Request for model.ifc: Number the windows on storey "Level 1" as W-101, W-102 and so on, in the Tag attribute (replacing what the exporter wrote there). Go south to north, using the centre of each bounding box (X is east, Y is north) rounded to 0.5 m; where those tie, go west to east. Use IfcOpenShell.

First a look at what the model holds.

```python
import ifcopenshell
import ifcopenshell.util.element
import ifcopenshell.util.placement

model = ifcopenshell.open("model.ifc")
print(model.schema)
storey = next(s for s in model.by_type("IfcBuildingStorey") if s.Name == "Level 1")
windows = [e for e in ifcopenshell.util.element.get_decomposition(storey) if e.is_a("IfcWindow")]
for e in sorted(windows, key=lambda e: e.id()):
    origin = ifcopenshell.util.placement.get_local_placement(e.ObjectPlacement)[:3, 3]
    print(e.id(), e.Tag, e.Name, origin.round(2) + 0.0, sep=" | ")
```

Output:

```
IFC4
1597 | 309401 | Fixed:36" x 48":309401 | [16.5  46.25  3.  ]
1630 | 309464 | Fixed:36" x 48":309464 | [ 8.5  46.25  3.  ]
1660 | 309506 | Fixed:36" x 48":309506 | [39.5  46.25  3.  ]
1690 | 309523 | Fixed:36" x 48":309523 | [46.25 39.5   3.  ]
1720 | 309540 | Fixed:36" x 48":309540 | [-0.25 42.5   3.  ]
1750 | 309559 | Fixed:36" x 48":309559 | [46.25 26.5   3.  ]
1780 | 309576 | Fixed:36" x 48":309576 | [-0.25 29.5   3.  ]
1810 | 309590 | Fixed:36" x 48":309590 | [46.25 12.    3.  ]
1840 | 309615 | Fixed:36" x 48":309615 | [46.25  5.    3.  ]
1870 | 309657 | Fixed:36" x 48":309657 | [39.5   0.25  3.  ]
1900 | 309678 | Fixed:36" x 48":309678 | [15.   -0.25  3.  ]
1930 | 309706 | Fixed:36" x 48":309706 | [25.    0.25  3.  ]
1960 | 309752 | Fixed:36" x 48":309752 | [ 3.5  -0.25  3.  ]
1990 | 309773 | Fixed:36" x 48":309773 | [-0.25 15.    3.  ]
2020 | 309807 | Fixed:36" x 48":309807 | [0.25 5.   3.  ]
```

```python
import ifcopenshell
import ifcopenshell.geom
import ifcopenshell.util.element
import ifcopenshell.util.shape

model = ifcopenshell.open("model.ifc")
settings = ifcopenshell.geom.settings()
settings.set("use-world-coords", True)


def centre(element):
    shape = ifcopenshell.geom.create_shape(settings, element)
    return ifcopenshell.util.shape.get_bbox_centroid(shape.geometry)


storey = next(s for s in model.by_type("IfcBuildingStorey") if s.Name == "Level 1")
windows = [e for e in ifcopenshell.util.element.get_decomposition(storey) if e.is_a("IfcWindow")]

# Insertion points can sit at a corner or the storey origin, so sort by the geometry (in metres).
centres = {e: centre(e) for e in windows}
windows.sort(key=lambda e: (round(centres[e][1] / 0.5), centres[e][0]))

for i, e in enumerate(windows, start=1):
    number = f"W-1{i:02d}"
    e.Tag = number
    print(e.id(), number)

model.write("model_edited.ifc")
```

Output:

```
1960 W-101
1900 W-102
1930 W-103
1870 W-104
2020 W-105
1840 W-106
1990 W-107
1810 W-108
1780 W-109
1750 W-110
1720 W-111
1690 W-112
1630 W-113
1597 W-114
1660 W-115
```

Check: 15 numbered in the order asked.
